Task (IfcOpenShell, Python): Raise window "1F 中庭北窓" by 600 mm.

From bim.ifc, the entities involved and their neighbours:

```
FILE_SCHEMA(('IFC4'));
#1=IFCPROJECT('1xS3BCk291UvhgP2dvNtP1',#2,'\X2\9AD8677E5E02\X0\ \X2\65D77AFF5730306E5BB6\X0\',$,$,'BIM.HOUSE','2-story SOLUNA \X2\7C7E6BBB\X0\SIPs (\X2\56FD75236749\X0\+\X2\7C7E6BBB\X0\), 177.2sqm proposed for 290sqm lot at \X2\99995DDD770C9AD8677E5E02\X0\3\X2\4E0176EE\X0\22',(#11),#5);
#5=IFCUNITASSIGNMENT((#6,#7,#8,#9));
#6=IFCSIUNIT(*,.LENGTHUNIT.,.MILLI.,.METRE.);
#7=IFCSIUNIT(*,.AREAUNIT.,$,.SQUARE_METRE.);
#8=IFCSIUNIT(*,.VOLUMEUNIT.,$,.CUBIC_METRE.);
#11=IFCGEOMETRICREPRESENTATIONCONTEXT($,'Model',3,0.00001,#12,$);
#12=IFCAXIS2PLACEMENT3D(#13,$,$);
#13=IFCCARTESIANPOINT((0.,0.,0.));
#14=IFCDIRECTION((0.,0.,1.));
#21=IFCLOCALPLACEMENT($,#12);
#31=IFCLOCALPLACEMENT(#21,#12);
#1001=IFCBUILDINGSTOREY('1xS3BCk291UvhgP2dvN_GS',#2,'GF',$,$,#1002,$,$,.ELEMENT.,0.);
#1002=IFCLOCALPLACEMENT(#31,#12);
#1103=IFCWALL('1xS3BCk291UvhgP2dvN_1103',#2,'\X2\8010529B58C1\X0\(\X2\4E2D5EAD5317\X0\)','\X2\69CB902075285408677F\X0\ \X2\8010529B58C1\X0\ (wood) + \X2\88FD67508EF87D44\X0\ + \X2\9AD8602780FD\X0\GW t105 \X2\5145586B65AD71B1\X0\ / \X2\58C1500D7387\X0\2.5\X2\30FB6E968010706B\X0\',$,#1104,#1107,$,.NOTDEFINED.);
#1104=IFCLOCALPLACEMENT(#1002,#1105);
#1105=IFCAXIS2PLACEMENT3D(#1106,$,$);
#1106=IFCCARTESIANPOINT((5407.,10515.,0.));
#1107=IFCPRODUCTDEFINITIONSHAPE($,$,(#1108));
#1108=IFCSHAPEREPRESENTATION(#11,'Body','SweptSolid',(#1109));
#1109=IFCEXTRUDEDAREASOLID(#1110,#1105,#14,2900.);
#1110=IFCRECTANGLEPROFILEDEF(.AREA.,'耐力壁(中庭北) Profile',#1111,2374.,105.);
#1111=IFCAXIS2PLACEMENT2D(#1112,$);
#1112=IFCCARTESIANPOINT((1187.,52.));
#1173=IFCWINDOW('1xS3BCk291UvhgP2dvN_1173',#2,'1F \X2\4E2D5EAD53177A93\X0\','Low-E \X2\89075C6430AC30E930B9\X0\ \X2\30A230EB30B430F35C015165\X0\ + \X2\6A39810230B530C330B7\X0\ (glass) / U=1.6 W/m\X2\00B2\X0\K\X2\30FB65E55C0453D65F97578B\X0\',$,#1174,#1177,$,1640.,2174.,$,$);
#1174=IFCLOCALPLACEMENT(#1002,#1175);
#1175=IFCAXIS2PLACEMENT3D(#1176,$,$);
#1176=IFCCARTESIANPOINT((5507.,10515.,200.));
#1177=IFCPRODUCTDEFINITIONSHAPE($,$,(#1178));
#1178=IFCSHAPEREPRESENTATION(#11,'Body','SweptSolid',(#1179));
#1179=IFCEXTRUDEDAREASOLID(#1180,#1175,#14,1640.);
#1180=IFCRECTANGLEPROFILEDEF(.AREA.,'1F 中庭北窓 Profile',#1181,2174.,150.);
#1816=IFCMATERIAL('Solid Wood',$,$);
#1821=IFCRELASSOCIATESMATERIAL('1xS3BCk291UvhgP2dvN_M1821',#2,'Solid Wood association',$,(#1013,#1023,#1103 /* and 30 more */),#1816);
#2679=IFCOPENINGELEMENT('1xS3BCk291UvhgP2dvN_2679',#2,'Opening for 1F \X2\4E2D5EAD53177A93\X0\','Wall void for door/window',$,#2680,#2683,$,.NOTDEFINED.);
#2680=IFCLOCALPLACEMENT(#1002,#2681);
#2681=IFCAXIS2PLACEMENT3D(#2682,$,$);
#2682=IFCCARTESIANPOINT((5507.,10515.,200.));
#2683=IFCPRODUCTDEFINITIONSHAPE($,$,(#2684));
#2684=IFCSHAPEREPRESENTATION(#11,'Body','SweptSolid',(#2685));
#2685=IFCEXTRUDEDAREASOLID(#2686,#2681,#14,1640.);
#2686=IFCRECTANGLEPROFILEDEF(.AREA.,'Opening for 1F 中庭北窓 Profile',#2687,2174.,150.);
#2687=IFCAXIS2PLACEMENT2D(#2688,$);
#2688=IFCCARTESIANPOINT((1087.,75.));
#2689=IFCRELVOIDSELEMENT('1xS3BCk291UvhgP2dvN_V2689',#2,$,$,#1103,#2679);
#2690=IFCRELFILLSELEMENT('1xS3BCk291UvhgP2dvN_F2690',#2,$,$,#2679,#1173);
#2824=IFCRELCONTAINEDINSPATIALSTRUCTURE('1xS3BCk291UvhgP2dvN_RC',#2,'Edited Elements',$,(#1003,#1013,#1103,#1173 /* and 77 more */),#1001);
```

```python
import numpy as np
import ifcopenshell
import ifcopenshell.api.geometry
import ifcopenshell.util.placement
import ifcopenshell.util.unit

model = ifcopenshell.open("bim.ifc")
unit_scale = ifcopenshell.util.unit.calculate_unit_scale(model)

window = model.by_guid("1xS3BCk291UvhgP2dvN_1173")
opening = window.FillsVoids[0].RelatingOpeningElement
dz = 0.6 / unit_scale

shift = np.array([0.0, 0.0, dz])
# The window is not placed relative to its opening, so move both.
for product in (opening, window):
    matrix = ifcopenshell.util.placement.get_local_placement(product.ObjectPlacement)
    matrix[:3, 3] += shift
    ifcopenshell.api.geometry.edit_object_placement(model, product=product, matrix=matrix, is_si=False)

print(f"moved by {dz * unit_scale:+.3f} m")

model.write("bim_edited.ifc")
```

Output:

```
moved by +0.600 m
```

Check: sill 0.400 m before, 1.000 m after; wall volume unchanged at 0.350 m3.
